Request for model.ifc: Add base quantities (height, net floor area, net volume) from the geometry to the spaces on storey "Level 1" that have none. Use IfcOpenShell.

First a look at what the model holds.

```python
import ifcopenshell
import ifcopenshell.util.element
import ifcopenshell.util.unit

model = ifcopenshell.open("model.ifc")
print(model.schema)
for unit_type in ("LENGTHUNIT", "AREAUNIT", "VOLUMEUNIT"):
    print(unit_type, ifcopenshell.util.unit.calculate_unit_scale(model, unit_type))
storey = next(s for s in model.by_type("IfcBuildingStorey") if s.Name == "Level 1")
spaces = [e for e in ifcopenshell.util.element.get_decomposition(storey) if e.is_a("IfcSpace")]
for e in sorted(spaces, key=lambda e: e.id()):
    print(e.id(), e.is_a(), e.Name, list(ifcopenshell.util.element.get_psets(e, qtos_only=True)), sep=" | ")
```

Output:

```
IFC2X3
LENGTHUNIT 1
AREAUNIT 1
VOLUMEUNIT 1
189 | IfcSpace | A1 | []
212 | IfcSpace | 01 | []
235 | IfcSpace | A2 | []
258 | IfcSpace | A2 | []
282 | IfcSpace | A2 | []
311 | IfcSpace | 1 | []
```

```python
import ifcopenshell
import ifcopenshell.api.pset
import ifcopenshell.geom
import ifcopenshell.util.element
import ifcopenshell.util.shape
import ifcopenshell.util.unit

model = ifcopenshell.open("model.ifc")
unit_scale = ifcopenshell.util.unit.calculate_unit_scale(model)
area_scale = ifcopenshell.util.unit.calculate_unit_scale(model, "AREAUNIT")
volume_scale = ifcopenshell.util.unit.calculate_unit_scale(model, "VOLUMEUNIT")
settings = ifcopenshell.geom.settings()

storey = next(s for s in model.by_type("IfcBuildingStorey") if s.Name == "Level 1")
spaces = [e for e in ifcopenshell.util.element.get_decomposition(storey) if e.is_a("IfcSpace")]

for e in sorted(spaces, key=lambda e: e.id()):
    if ifcopenshell.util.element.get_psets(e, qtos_only=True, should_inherit=False):
        continue
    # Geometry comes back in metres, in the element's own axes.
    shape = ifcopenshell.geom.create_shape(settings, e)
    values = {
        "Height": ifcopenshell.util.shape.get_z(shape.geometry) / unit_scale,
        "NetFloorArea": ifcopenshell.util.shape.get_footprint_area(shape.geometry) / area_scale,
        "NetVolume": ifcopenshell.util.shape.get_volume(shape.geometry) / volume_scale,
    }
    qto = ifcopenshell.api.pset.add_qto(model, product=e, name="BaseQuantities")
    ifcopenshell.api.pset.edit_qto(model, qto=qto, properties=values)
    print(e.id(), {k: round(v, 3) for k, v in values.items()})

model.write("model_updated.ifc")
```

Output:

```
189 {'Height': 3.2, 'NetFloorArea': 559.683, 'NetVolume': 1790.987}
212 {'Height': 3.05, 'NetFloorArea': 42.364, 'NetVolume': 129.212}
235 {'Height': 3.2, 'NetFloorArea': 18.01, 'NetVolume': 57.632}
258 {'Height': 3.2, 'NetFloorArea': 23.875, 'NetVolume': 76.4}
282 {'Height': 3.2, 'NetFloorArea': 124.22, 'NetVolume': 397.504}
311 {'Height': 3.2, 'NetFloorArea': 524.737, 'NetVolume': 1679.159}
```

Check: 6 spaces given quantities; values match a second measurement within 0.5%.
